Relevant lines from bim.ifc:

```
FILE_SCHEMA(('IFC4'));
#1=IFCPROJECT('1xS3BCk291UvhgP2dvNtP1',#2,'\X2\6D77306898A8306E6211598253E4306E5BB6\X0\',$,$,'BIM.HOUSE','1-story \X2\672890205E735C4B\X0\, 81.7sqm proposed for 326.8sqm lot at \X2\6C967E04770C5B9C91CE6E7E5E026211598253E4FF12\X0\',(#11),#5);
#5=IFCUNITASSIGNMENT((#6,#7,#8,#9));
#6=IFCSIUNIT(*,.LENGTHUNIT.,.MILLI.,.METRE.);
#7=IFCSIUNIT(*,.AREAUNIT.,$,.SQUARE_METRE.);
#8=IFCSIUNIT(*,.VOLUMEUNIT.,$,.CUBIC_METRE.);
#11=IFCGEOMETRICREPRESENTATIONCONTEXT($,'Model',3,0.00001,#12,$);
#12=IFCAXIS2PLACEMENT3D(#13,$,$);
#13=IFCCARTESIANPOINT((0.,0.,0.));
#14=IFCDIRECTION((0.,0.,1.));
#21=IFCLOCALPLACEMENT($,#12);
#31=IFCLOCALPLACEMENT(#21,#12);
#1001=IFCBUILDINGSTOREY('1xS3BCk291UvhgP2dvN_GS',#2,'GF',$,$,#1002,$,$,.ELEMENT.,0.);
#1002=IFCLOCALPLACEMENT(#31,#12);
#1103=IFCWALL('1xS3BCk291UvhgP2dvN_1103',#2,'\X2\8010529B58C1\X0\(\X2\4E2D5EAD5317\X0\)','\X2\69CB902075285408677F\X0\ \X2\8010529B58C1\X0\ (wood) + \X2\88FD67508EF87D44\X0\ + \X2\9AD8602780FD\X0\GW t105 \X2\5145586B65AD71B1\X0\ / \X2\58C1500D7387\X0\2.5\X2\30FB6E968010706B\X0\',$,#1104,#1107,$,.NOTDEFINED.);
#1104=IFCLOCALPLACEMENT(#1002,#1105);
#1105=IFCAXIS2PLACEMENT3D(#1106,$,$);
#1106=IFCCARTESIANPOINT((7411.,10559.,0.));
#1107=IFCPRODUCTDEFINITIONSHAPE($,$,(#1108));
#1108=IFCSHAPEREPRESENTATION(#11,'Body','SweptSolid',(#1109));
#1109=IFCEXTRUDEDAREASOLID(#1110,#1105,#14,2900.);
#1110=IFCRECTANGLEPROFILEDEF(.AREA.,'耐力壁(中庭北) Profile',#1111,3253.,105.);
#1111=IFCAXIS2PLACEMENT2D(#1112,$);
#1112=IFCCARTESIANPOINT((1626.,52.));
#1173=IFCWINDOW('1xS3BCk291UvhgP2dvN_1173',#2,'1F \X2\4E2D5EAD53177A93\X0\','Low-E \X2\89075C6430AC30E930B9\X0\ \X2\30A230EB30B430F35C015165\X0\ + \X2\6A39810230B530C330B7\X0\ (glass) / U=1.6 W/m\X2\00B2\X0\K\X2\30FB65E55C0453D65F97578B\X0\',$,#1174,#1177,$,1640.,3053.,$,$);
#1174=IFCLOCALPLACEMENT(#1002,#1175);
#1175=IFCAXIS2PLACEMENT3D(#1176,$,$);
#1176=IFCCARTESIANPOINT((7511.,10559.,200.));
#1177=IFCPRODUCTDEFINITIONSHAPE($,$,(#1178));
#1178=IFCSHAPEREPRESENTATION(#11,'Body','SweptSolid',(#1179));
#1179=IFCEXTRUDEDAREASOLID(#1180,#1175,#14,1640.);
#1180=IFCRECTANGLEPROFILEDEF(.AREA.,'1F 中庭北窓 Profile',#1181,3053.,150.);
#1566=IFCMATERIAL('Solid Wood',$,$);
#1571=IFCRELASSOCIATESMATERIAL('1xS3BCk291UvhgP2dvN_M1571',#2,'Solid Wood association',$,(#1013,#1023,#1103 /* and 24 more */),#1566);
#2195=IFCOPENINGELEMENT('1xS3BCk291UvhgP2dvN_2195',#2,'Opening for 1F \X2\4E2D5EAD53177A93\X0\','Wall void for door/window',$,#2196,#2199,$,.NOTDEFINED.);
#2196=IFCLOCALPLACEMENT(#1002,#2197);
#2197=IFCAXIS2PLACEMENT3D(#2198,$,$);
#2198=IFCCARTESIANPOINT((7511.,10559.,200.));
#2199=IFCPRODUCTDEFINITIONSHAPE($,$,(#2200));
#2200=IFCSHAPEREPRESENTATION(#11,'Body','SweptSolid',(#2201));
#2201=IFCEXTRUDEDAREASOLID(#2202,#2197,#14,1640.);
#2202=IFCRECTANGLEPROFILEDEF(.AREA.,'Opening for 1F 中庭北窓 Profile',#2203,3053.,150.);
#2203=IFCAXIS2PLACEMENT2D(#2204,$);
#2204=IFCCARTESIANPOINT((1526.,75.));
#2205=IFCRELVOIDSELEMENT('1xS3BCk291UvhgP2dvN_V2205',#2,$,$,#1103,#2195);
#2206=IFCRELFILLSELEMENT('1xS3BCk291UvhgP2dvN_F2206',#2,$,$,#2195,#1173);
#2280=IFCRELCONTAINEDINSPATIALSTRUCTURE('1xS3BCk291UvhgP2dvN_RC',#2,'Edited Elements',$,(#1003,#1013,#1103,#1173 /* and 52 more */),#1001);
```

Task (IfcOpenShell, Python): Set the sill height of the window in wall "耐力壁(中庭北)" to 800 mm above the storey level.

```python
import numpy as np
import ifcopenshell
import ifcopenshell.api.geometry
import ifcopenshell.geom
import ifcopenshell.util.element
import ifcopenshell.util.placement
import ifcopenshell.util.shape
import ifcopenshell.util.unit

model = ifcopenshell.open("bim.ifc")
unit_scale = ifcopenshell.util.unit.calculate_unit_scale(model)

window = model.by_guid("1xS3BCk291UvhgP2dvN_1173")
opening = window.FillsVoids[0].RelatingOpeningElement
storey = ifcopenshell.util.element.get_container(window, ifc_class="IfcBuildingStorey")
level = ifcopenshell.util.placement.get_local_placement(storey.ObjectPlacement)[2, 3]

# The opening's origin need not be at the sill, so measure its lowest point.
shape = ifcopenshell.geom.create_shape(ifcopenshell.geom.settings(), opening)
bottom = ifcopenshell.util.shape.get_shape_bottom_elevation(shape, shape.geometry) / unit_scale
dz = level + 800.0 - bottom

shift = np.array([0.0, 0.0, dz])
# The window is not placed relative to its opening, so move both.
for product in (opening, window):
    matrix = ifcopenshell.util.placement.get_local_placement(product.ObjectPlacement)
    matrix[:3, 3] += shift
    ifcopenshell.api.geometry.edit_object_placement(model, product=product, matrix=matrix, is_si=False)

print(f"moved by {dz * unit_scale:+.3f} m")

model.write("bim_rev.ifc")
```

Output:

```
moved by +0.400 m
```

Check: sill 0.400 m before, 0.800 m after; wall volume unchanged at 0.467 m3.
